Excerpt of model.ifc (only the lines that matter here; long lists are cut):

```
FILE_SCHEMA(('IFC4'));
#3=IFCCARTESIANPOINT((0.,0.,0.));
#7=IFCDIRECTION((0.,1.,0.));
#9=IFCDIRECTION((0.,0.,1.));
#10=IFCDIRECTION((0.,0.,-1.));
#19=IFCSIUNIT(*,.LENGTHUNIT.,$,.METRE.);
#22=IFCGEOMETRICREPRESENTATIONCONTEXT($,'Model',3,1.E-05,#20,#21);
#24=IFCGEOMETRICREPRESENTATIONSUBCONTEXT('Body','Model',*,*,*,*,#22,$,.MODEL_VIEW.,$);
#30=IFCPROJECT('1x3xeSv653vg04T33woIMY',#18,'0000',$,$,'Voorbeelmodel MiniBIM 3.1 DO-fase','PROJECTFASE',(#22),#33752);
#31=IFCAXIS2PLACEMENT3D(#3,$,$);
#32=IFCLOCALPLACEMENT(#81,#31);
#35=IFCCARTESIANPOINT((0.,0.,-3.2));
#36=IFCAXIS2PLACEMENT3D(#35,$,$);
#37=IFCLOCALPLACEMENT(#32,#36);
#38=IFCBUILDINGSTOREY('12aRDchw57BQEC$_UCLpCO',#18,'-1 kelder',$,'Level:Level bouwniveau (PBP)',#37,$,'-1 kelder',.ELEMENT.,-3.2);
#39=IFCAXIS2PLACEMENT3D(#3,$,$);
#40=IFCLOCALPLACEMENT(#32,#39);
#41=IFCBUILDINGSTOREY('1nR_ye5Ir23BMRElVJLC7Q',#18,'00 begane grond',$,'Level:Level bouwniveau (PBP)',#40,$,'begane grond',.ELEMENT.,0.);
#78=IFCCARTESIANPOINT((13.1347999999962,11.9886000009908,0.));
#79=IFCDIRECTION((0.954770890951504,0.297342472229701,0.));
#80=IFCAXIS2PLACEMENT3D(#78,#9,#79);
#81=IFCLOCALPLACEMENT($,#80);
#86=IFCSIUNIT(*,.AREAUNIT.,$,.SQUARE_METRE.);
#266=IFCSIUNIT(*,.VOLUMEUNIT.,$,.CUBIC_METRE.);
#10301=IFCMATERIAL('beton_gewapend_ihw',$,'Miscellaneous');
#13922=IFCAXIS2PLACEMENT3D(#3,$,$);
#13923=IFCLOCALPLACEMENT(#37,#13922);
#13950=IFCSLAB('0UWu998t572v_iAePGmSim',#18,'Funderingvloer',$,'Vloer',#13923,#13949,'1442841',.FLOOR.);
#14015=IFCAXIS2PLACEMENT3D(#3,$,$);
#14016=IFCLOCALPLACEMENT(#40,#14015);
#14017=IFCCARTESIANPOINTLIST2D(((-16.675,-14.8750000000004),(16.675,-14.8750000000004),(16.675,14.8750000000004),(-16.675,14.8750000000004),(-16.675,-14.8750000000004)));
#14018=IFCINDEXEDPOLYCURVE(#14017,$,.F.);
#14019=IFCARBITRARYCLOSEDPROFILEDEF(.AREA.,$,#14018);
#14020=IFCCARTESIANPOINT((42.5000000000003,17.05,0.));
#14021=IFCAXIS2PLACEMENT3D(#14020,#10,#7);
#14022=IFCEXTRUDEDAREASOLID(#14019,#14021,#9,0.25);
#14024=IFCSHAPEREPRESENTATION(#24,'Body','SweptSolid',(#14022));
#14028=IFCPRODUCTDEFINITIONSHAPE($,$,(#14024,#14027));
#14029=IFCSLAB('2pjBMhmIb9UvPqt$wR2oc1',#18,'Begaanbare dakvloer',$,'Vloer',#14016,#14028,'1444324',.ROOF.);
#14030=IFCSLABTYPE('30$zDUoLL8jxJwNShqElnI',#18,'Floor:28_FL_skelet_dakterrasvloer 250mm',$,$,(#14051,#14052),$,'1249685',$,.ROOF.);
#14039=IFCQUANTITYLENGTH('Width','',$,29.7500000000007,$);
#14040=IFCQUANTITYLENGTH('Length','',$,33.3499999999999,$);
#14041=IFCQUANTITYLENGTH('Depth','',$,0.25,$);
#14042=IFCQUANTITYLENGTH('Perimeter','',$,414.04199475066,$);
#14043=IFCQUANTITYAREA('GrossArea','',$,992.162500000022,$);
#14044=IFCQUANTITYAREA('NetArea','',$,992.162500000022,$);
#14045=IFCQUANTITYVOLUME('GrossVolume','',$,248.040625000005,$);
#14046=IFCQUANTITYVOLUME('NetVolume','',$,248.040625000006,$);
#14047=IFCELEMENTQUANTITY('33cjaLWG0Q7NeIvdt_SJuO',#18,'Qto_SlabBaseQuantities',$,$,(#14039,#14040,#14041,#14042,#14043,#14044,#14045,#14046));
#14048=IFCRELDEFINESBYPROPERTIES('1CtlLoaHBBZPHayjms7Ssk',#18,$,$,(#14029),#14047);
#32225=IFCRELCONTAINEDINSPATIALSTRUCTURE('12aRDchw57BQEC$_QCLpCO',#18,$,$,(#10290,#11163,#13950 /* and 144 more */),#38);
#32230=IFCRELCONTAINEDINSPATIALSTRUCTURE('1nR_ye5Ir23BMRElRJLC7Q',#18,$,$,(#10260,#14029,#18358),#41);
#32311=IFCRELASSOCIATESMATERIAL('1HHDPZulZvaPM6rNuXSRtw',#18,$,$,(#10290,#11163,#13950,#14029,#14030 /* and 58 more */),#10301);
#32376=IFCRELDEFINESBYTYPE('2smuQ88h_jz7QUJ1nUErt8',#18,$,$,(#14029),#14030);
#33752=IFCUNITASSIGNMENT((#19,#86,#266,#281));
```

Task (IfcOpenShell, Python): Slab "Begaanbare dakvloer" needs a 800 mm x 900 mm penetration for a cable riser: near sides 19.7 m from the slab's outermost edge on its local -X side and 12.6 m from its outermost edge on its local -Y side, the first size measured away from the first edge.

```python
import numpy as np
import ifcopenshell
import ifcopenshell.api.feature
import ifcopenshell.api.geometry
import ifcopenshell.api.pset
import ifcopenshell.api.root
import ifcopenshell.geom
import ifcopenshell.util.element
import ifcopenshell.util.placement
import ifcopenshell.util.representation
import ifcopenshell.util.shape
import ifcopenshell.util.unit

model = ifcopenshell.open("model.ifc")
unit_scale = ifcopenshell.util.unit.calculate_unit_scale(model)
area_scale = ifcopenshell.util.unit.calculate_unit_scale(model, "AREAUNIT")
volume_scale = ifcopenshell.util.unit.calculate_unit_scale(model, "VOLUMEUNIT")
settings = ifcopenshell.geom.settings()


def volume(element):
    """Net volume in cubic metres, openings subtracted."""
    shape = ifcopenshell.geom.create_shape(settings, element)
    return ifcopenshell.util.shape.get_volume(shape.geometry)


slab = model.by_guid("2pjBMhmIb9UvPqt$wR2oc1")
before = volume(slab)

# Extent in the slab's own axes, in metres. The edges named are its -X and -Y sides.
slab_shape = ifcopenshell.geom.create_shape(settings, slab)
vertices = ifcopenshell.util.shape.get_vertices(slab_shape.geometry)
x_min, y_min, bottom = vertices.min(axis=0)
top = vertices[:, 2].max()

opening = ifcopenshell.api.root.create_entity(model, ifc_class="IfcOpeningElement", name="Cable riser opening", predefined_type="OPENING")
context = ifcopenshell.util.representation.get_context(model, "Model", "Body", "MODEL_VIEW")
width, depth = 0.8, 0.9
outline = [(0.0, 0.0), (width, 0.0), (width, depth), (0.0, depth), (0.0, 0.0)]
# Overshoot both faces by 50 mm so the cut is clean.
shape = ifcopenshell.api.geometry.add_slab_representation(
    model, context=context, depth=top - bottom + 0.1, polyline=outline
)
ifcopenshell.api.geometry.assign_representation(model, product=opening, representation=shape)

matrix = ifcopenshell.util.placement.get_local_placement(slab.ObjectPlacement)
matrix[:, 3] = matrix @ np.append(np.array([x_min + 19.7, y_min + 12.6, bottom - 0.05]) / unit_scale, 1.0)
ifcopenshell.api.geometry.edit_object_placement(model, product=opening, matrix=matrix, is_si=False)
ifcopenshell.api.feature.add_feature(model, feature=opening, element=slab)

after = volume(slab)

# Update the slab's stored quantities.
qto = model.by_id(ifcopenshell.util.element.get_pset(slab, "Qto_SlabBaseQuantities", should_inherit=False)["id"])
ifcopenshell.api.pset.edit_qto(model, qto=qto, properties={
    "NetArea": after / (top - bottom) / area_scale,
    "NetVolume": after / volume_scale,
})

print(f"slab volume {before:.3f} -> {after:.3f} m3")

model.write("model-out.ifc")
```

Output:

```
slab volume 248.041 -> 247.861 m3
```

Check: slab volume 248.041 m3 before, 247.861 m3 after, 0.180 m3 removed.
